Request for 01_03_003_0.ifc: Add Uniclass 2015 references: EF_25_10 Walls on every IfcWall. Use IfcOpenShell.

First a look at what the model holds.

```python
import ifcopenshell

model = ifcopenshell.open("01_03_003_0.ifc")
print(model.schema)
print("classifications:", [c.Name for c in model.by_type("IfcClassification")])
for ifc_class in ("IfcDoor", "IfcRoof", "IfcStair", "IfcWall", "IfcWindow"):
    print(ifc_class, len(model.by_type(ifc_class)))
```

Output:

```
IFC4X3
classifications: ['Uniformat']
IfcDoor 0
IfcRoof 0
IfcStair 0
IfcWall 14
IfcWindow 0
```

```python
import ifcopenshell
import ifcopenshell.api.classification

model = ifcopenshell.open("01_03_003_0.ifc")

system = ifcopenshell.api.classification.add_classification(model, classification="Uniclass 2015")

codes = {
    "IfcWall": ("EF_25_10", "Walls"),
}
for ifc_class, (code, name) in codes.items():
    products = model.by_type(ifc_class)
    ifcopenshell.api.classification.add_reference(
        model, products=products, classification=system, identification=code, name=name
    )
    print(code, len(products))

model.write("01_03_003_0-out.ifc")
```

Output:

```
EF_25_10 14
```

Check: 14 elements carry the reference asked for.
